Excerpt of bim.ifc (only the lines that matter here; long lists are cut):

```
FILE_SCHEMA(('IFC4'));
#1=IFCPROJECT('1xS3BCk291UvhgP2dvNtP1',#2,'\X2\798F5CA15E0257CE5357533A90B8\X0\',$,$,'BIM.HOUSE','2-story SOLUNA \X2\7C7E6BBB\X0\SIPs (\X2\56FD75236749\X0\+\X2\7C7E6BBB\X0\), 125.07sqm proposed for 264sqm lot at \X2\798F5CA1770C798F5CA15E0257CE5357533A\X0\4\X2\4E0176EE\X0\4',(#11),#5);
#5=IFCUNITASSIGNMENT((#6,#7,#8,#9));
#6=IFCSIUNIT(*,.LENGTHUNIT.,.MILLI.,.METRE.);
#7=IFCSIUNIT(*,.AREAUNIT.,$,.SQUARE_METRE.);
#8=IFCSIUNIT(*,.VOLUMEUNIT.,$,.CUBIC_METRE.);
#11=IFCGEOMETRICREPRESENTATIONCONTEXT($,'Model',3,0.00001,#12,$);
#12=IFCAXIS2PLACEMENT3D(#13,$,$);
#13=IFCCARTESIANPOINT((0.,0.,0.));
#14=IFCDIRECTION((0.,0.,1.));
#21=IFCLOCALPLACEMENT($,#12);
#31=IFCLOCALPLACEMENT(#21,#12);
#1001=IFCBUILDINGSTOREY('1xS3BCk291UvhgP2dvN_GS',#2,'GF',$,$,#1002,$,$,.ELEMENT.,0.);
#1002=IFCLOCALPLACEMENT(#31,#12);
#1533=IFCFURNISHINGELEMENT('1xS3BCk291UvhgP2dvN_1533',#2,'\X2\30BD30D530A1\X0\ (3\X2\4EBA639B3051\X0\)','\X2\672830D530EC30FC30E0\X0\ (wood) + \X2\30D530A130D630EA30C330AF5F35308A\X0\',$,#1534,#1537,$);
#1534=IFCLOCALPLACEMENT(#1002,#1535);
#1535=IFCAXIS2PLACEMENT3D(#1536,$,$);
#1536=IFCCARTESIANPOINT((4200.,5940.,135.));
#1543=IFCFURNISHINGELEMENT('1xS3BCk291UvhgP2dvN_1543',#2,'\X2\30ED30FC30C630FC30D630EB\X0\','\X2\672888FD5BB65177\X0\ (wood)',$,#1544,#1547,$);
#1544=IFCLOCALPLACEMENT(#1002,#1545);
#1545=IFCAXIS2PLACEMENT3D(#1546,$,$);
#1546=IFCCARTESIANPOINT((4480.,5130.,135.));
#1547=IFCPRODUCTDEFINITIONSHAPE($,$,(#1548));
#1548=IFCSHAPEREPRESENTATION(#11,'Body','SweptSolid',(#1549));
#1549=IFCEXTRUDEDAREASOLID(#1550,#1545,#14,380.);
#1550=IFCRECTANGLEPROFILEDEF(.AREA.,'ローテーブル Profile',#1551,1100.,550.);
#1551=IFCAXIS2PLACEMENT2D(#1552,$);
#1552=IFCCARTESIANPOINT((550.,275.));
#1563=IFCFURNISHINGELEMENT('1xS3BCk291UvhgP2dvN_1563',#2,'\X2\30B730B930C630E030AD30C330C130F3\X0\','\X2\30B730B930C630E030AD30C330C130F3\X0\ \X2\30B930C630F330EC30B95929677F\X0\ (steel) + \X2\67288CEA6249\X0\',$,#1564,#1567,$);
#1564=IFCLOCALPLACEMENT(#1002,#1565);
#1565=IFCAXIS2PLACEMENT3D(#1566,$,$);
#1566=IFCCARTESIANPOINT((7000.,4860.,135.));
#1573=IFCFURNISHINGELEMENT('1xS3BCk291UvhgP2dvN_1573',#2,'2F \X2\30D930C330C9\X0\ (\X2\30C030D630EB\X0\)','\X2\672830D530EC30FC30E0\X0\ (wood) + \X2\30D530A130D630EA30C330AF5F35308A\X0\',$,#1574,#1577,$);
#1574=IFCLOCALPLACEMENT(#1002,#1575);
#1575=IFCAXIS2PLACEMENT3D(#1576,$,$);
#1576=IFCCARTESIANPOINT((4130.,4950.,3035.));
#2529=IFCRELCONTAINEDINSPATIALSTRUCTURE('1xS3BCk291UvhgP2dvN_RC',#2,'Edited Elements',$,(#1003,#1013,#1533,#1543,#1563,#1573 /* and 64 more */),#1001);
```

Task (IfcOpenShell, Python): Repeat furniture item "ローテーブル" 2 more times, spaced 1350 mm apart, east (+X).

```python
import numpy as np
import ifcopenshell
import ifcopenshell.api.geometry
import ifcopenshell.api.root
import ifcopenshell.util.element
import ifcopenshell.util.placement

model = ifcopenshell.open("bim.ifc")


def reuse_history(source, copy):
    """copy_class also copies each property set's owner history, people and application; keep the originals."""
    for rel in copy.IsDefinedBy:
        if rel.is_a("IfcRelDefinesByProperties") and (history := rel.RelatingPropertyDefinition.OwnerHistory):
            rel.RelatingPropertyDefinition.OwnerHistory = source.OwnerHistory
            ifcopenshell.util.element.remove_deep2(model, history)


source = model.by_guid("1xS3BCk291UvhgP2dvN_1543")
base = ifcopenshell.util.placement.get_local_placement(source.ObjectPlacement)
step = np.array([1.0, 0.0, 0.0]) * 1350.0

for i in range(1, 3):
    copy = ifcopenshell.api.root.copy_class(model, product=source)
    copy.Representation = ifcopenshell.util.element.copy_deep(
        model, source.Representation, exclude=["IfcGeometricRepresentationContext", "IfcRepresentationMap"]
    )
    reuse_history(source, copy)
    matrix = base.copy()
    matrix[:3, 3] += i * step
    print("added at", matrix[:3, 3].round(3) + 0.0)
    ifcopenshell.api.geometry.edit_object_placement(model, product=copy, matrix=matrix, is_si=False)

model.write("bim_v2.ifc")
```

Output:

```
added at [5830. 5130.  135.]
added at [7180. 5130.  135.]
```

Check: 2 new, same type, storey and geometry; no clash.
